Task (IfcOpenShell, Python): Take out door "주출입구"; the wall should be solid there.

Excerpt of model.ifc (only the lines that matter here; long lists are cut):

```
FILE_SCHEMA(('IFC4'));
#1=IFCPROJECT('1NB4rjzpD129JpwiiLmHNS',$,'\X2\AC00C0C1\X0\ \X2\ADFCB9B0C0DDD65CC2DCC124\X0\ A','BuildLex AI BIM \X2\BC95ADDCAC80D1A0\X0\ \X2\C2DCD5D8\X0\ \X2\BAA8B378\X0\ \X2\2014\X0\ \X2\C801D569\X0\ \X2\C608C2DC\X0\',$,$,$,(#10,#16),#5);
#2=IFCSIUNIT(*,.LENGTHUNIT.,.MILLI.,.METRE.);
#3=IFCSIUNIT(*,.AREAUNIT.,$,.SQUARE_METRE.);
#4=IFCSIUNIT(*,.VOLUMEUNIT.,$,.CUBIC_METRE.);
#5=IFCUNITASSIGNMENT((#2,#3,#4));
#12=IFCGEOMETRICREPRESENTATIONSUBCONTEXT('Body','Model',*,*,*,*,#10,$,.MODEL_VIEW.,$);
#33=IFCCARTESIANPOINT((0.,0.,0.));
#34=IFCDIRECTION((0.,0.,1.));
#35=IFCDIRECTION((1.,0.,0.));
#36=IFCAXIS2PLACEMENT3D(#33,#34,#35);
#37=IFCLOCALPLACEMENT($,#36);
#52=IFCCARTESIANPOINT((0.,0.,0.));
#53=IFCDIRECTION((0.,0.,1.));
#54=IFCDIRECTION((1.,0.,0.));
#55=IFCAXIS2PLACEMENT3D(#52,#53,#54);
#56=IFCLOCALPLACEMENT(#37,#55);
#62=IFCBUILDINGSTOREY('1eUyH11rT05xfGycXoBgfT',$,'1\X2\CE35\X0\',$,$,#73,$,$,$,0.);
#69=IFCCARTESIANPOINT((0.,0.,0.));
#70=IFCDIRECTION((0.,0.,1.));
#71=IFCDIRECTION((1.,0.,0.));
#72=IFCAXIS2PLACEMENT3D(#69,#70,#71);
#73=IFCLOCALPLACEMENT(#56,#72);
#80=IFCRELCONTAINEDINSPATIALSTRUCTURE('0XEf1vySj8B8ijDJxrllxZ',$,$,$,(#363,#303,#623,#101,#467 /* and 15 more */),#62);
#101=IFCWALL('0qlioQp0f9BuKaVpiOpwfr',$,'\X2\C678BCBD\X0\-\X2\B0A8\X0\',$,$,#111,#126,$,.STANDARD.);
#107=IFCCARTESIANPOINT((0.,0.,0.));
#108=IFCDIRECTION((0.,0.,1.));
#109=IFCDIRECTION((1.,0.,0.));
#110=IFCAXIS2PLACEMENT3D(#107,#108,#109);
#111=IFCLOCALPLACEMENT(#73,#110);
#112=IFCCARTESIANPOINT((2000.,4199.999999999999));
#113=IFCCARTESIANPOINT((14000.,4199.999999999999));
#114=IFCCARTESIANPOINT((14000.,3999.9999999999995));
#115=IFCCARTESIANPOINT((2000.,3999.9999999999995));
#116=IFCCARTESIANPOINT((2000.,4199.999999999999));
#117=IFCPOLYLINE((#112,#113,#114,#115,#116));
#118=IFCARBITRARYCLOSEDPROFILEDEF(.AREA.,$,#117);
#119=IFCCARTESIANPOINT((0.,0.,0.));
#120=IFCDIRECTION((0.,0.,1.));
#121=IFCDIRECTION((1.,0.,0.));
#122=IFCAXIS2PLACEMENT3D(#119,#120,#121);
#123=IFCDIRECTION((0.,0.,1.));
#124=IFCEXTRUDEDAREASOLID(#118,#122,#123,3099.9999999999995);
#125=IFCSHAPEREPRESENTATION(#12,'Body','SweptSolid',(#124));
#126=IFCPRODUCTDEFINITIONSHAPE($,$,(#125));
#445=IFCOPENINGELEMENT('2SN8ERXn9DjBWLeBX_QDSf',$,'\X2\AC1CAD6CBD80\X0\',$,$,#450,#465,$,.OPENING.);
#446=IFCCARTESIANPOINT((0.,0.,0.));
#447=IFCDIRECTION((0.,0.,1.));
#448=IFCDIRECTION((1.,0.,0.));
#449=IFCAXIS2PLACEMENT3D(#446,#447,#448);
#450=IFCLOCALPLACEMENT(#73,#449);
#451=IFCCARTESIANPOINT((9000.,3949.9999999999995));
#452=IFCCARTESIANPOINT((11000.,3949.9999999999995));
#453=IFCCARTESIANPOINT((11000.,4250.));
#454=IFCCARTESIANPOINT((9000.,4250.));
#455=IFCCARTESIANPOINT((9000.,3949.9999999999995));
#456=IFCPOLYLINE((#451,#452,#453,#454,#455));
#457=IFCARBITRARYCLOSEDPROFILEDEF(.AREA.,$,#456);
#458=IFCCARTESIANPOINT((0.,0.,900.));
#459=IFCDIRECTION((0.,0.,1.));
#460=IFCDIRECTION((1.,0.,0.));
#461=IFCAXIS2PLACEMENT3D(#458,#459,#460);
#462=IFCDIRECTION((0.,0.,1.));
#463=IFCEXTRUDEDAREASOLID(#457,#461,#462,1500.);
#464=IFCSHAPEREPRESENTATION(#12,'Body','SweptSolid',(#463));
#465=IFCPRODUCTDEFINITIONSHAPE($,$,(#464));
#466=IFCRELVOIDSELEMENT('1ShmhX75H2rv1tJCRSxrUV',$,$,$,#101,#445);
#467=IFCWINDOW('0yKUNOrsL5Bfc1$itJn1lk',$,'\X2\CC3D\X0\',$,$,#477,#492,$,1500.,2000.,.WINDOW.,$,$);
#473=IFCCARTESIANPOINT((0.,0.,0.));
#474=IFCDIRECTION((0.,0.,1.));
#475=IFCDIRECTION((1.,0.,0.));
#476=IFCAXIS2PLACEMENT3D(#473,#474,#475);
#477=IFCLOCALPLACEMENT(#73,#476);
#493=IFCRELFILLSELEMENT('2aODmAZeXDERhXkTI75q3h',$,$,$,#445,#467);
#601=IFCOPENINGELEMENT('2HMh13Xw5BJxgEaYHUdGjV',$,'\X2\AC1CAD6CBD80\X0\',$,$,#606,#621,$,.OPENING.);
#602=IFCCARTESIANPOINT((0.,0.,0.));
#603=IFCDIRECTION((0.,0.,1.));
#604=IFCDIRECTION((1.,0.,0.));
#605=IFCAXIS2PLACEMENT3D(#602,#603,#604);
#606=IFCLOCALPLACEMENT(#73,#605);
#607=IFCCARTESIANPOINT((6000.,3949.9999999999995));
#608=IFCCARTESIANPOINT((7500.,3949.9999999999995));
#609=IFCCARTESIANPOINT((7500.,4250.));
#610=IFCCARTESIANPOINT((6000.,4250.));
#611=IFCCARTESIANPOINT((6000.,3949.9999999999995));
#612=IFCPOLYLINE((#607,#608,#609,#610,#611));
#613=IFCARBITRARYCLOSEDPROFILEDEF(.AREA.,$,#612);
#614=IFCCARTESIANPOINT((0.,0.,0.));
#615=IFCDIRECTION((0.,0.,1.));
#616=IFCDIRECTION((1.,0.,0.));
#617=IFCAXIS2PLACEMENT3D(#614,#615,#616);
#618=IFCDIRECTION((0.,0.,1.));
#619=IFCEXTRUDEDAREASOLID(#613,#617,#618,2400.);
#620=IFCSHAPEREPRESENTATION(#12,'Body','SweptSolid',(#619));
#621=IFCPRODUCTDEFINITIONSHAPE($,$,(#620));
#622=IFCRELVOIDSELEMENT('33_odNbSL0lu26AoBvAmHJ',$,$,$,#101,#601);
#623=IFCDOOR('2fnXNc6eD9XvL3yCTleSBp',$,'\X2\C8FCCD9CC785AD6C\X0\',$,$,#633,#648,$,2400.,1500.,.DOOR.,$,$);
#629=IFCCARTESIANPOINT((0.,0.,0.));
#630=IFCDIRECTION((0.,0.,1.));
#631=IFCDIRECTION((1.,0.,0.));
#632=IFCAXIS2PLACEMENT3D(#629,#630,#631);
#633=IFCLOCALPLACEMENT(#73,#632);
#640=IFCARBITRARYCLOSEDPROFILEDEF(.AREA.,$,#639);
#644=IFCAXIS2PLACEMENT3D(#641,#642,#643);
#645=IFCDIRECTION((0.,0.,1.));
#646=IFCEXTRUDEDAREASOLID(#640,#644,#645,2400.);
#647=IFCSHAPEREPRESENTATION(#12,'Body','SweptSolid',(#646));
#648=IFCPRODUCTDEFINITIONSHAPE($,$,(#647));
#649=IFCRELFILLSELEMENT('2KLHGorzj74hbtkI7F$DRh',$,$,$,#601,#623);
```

```python
import ifcopenshell
import ifcopenshell.api.feature
import ifcopenshell.api.root
import ifcopenshell.geom
import ifcopenshell.util.shape

model = ifcopenshell.open("model.ifc")
settings = ifcopenshell.geom.settings()


def volume(element):
    """Net volume in cubic metres, openings subtracted."""
    shape = ifcopenshell.geom.create_shape(settings, element)
    return ifcopenshell.util.shape.get_volume(shape.geometry)


door = model.by_id(623)
opening = door.FillsVoids[0].RelatingOpeningElement
wall = opening.VoidsElements[0].RelatingBuildingElement
before = volume(wall)

ifcopenshell.api.root.remove_product(model, product=door)
ifcopenshell.api.feature.remove_feature(model, feature=opening)

after = volume(wall)

print(f"wall volume {before:.3f} -> {after:.3f} m3")

model.write("model_updated.ifc")
```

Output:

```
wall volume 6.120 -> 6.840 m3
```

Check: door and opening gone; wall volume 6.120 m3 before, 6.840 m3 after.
